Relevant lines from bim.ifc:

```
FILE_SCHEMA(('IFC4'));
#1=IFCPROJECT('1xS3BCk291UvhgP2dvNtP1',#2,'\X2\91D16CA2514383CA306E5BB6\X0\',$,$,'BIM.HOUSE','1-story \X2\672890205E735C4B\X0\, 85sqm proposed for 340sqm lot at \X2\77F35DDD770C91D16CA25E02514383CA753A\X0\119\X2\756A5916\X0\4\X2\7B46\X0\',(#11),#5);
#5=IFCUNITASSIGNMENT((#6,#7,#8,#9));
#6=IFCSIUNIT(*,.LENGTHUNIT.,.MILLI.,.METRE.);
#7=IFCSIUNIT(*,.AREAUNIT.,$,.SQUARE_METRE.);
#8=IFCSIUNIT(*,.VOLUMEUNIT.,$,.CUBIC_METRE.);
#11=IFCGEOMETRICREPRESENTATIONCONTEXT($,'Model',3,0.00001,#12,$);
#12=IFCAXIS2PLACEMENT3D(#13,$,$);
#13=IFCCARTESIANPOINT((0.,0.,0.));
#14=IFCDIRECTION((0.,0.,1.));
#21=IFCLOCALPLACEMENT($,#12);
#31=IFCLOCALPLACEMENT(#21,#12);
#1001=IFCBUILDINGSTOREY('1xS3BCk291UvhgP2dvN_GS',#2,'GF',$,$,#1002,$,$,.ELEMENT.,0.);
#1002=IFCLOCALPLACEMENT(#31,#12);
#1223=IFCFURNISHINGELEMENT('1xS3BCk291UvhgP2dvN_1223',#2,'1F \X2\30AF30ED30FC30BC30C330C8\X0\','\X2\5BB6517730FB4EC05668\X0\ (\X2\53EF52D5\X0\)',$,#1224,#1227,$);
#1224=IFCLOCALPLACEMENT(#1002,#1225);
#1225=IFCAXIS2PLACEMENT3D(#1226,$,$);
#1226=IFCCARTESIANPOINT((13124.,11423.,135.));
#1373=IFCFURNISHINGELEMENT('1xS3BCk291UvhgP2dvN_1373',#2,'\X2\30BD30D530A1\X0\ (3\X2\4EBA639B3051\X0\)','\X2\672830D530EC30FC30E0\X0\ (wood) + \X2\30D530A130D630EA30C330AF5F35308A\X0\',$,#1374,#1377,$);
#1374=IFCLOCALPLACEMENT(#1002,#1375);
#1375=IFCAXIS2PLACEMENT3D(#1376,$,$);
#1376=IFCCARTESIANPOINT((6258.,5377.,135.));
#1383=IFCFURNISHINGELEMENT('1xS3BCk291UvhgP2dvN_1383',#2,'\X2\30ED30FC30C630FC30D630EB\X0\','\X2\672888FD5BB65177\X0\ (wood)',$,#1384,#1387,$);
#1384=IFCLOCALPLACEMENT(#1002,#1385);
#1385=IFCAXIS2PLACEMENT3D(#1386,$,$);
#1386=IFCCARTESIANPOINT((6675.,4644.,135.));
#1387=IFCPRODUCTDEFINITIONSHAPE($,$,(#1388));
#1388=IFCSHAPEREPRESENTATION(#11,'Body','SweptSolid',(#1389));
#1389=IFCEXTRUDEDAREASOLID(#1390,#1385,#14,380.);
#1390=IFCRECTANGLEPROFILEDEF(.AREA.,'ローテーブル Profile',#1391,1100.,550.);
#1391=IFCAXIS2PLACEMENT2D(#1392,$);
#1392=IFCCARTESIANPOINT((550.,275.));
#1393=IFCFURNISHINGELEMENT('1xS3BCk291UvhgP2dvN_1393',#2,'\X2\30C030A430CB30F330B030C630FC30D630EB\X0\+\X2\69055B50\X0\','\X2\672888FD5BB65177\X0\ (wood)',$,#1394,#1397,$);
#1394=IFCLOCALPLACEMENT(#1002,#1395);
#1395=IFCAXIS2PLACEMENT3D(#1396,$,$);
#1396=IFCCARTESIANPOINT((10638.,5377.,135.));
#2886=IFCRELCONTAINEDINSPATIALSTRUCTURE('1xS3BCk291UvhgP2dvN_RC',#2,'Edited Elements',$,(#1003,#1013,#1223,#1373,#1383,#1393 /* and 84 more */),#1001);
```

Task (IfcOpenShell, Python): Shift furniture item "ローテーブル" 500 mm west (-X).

```python
import ifcopenshell
import ifcopenshell.api.geometry
import ifcopenshell.util.placement
import ifcopenshell.util.unit

model = ifcopenshell.open("bim.ifc")
unit_scale = ifcopenshell.util.unit.calculate_unit_scale(model)

item = model.by_guid("1xS3BCk291UvhgP2dvN_1383")
matrix = ifcopenshell.util.placement.get_local_placement(item.ObjectPlacement)
matrix[0, 3] -= 0.5 / unit_scale
ifcopenshell.api.geometry.edit_object_placement(model, product=item, matrix=matrix, is_si=False)

print(ifcopenshell.util.placement.get_local_placement(item.ObjectPlacement).round(3) + 0.0)

model.write("bim-out.ifc")
```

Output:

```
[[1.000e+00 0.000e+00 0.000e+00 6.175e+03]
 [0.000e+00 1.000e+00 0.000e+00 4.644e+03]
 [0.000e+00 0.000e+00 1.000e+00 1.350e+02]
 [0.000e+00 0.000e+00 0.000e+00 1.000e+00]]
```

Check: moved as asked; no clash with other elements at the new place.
